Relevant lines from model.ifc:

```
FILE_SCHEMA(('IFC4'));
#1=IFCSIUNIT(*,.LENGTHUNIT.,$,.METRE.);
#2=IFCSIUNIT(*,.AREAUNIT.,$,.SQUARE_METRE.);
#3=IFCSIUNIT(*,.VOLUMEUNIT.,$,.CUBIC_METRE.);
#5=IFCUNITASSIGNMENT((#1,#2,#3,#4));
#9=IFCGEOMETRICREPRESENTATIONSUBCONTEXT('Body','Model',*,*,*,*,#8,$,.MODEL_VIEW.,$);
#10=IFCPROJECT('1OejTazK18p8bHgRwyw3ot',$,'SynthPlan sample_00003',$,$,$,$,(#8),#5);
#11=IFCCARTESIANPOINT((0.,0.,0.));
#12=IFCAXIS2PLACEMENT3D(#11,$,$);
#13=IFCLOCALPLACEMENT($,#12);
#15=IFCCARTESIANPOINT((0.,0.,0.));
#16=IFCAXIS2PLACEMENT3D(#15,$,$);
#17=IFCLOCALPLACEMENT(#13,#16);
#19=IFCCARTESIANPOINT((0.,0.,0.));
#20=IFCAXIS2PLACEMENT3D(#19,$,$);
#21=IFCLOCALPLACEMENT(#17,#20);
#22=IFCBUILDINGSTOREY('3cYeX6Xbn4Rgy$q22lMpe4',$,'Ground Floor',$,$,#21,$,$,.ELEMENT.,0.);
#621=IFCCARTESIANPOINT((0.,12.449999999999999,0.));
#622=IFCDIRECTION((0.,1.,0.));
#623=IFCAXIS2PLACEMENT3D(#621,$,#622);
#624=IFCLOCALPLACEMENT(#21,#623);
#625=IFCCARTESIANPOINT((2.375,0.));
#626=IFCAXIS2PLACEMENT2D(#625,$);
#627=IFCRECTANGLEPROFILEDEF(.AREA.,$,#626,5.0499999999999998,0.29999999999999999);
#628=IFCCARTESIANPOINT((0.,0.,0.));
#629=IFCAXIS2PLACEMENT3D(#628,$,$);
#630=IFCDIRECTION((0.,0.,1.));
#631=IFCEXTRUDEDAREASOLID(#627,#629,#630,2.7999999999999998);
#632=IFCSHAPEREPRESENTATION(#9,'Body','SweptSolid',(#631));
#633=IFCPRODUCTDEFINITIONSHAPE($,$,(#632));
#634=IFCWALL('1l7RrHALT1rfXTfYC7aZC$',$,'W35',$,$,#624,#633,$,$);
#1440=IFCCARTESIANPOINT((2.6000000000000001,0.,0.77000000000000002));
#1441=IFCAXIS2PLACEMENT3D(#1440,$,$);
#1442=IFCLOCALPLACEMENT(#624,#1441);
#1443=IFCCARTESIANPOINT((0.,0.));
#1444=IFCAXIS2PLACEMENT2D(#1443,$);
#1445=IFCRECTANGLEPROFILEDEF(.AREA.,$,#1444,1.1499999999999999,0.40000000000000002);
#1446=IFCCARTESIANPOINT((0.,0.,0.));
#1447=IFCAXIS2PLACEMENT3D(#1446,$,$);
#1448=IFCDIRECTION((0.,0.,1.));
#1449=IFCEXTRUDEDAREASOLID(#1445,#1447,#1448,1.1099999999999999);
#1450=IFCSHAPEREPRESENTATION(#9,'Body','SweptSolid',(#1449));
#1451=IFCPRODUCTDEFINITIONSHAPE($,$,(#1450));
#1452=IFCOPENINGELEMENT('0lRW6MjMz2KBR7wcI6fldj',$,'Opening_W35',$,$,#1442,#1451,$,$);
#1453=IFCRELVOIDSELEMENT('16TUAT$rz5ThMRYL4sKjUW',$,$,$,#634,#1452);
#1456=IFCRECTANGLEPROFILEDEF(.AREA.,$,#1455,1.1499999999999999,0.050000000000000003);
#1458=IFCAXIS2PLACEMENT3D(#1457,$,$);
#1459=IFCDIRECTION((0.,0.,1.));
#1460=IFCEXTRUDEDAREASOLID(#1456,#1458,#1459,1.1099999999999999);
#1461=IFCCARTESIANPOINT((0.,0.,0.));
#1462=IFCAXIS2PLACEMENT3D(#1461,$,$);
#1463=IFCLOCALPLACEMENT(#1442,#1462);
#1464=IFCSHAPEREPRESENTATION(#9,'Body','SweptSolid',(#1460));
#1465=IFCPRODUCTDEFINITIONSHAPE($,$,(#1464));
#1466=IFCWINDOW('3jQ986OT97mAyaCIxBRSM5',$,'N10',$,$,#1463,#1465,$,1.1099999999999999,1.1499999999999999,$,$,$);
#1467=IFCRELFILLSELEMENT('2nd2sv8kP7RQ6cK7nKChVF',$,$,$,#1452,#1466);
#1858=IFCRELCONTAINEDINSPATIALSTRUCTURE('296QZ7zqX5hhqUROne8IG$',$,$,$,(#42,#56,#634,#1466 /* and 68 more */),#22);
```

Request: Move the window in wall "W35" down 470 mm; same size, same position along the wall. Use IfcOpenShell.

```python
import numpy as np
import ifcopenshell
import ifcopenshell.api.geometry
import ifcopenshell.util.placement
import ifcopenshell.util.unit

model = ifcopenshell.open("model.ifc")
unit_scale = ifcopenshell.util.unit.calculate_unit_scale(model)

window = model.by_id(1466)
opening = window.FillsVoids[0].RelatingOpeningElement
dz = -0.47 / unit_scale

shift = np.array([0.0, 0.0, dz])
# The window is placed relative to its opening, so it follows when the opening moves.
matrix = ifcopenshell.util.placement.get_local_placement(opening.ObjectPlacement)
matrix[:3, 3] += shift
ifcopenshell.api.geometry.edit_object_placement(
    model, product=opening, matrix=matrix, is_si=False, should_transform_children=True
)

print(f"moved by {dz * unit_scale:+.3f} m")

model.write("model-out.ifc")
```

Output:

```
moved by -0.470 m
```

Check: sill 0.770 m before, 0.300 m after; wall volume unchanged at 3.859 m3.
